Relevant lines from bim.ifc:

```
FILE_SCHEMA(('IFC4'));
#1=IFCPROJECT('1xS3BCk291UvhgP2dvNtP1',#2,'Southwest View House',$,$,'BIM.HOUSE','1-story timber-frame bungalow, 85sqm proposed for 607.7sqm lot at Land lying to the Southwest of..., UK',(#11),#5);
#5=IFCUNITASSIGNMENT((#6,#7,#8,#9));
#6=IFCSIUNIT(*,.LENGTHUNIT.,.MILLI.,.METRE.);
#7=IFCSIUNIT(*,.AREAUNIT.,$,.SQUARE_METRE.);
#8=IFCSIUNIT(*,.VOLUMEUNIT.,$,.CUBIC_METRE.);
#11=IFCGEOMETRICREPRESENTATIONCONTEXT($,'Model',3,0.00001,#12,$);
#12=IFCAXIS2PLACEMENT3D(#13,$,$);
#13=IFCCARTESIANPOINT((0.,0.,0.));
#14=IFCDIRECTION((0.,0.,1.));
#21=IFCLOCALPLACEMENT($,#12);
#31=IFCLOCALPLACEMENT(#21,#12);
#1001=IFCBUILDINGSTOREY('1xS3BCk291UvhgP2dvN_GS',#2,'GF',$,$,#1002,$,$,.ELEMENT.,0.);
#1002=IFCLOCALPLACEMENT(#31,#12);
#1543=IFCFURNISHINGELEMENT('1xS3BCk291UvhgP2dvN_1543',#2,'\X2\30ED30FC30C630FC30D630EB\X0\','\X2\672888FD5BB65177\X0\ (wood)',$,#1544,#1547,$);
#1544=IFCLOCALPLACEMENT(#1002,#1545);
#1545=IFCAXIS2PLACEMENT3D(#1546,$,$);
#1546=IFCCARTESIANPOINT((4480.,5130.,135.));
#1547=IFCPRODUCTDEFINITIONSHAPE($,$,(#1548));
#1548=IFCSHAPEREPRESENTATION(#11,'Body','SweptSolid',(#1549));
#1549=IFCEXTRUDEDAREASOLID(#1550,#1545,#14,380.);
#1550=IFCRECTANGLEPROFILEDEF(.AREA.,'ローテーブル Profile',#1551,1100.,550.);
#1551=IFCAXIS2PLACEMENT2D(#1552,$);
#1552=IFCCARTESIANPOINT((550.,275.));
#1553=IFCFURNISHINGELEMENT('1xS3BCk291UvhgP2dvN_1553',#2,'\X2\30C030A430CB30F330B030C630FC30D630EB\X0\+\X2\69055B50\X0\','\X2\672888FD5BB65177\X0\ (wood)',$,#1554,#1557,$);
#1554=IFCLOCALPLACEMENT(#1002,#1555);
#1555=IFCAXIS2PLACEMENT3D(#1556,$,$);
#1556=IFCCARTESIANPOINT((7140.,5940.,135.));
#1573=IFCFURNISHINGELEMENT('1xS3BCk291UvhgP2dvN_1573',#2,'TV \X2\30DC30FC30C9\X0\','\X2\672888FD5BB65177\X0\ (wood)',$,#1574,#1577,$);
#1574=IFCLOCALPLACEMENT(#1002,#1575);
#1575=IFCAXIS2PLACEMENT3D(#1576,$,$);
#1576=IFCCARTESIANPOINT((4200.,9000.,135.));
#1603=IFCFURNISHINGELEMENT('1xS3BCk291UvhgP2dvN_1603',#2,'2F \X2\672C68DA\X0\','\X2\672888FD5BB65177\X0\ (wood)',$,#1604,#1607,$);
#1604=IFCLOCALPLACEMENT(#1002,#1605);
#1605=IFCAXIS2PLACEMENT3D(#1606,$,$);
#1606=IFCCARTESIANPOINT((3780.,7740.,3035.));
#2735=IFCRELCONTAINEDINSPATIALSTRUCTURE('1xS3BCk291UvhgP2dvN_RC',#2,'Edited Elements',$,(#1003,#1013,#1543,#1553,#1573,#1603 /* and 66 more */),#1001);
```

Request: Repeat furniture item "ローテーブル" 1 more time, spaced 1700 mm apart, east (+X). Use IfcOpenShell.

```python
import numpy as np
import ifcopenshell
import ifcopenshell.api.geometry
import ifcopenshell.api.root
import ifcopenshell.util.element
import ifcopenshell.util.placement
import ifcopenshell.util.unit

model = ifcopenshell.open("bim.ifc")
unit_scale = ifcopenshell.util.unit.calculate_unit_scale(model)


def reuse_history(source, copy):
    """copy_class also copies each property set's owner history, people and application; keep the originals."""
    for rel in copy.IsDefinedBy:
        if rel.is_a("IfcRelDefinesByProperties") and (history := rel.RelatingPropertyDefinition.OwnerHistory):
            rel.RelatingPropertyDefinition.OwnerHistory = source.OwnerHistory
            ifcopenshell.util.element.remove_deep2(model, history)


source = model.by_id(1543)
base = ifcopenshell.util.placement.get_local_placement(source.ObjectPlacement)
step = np.array([1.0, 0.0, 0.0]) * 1.7 / unit_scale

for i in range(1, 2):
    copy = ifcopenshell.api.root.copy_class(model, product=source)
    copy.Representation = ifcopenshell.util.element.copy_deep(
        model, source.Representation, exclude=["IfcGeometricRepresentationContext", "IfcRepresentationMap"]
    )
    reuse_history(source, copy)
    matrix = base.copy()
    matrix[:3, 3] += i * step
    print("added at", matrix[:3, 3].round(3) + 0.0)
    ifcopenshell.api.geometry.edit_object_placement(model, product=copy, matrix=matrix, is_si=False)

model.write("bim_edited.ifc")
```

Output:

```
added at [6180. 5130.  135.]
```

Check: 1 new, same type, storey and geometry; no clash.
